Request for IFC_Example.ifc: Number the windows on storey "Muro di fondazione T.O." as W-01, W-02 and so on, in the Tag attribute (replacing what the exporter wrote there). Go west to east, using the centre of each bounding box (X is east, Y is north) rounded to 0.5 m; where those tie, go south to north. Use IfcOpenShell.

First a look at what the model holds.

```python
import ifcopenshell
import ifcopenshell.util.element
import ifcopenshell.util.placement

model = ifcopenshell.open("IFC_Example.ifc")
print(model.schema)
storey = next(s for s in model.by_type("IfcBuildingStorey") if s.Name == "Muro di fondazione T.O.")
windows = [e for e in ifcopenshell.util.element.get_decomposition(storey) if e.is_a("IfcWindow")]
for e in sorted(windows, key=lambda e: e.id()):
    origin = ifcopenshell.util.placement.get_local_placement(e.ObjectPlacement)[:3, 3]
    print(e.id(), e.Tag, e.Name, origin.round(2) + 0.0, sep=" | ")
```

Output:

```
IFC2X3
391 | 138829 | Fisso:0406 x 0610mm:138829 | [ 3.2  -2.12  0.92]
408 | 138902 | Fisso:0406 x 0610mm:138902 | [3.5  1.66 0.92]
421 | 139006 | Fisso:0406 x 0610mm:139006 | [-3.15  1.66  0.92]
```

```python
import ifcopenshell
import ifcopenshell.geom
import ifcopenshell.util.element
import ifcopenshell.util.shape

model = ifcopenshell.open("IFC_Example.ifc")
settings = ifcopenshell.geom.settings()
settings.set("use-world-coords", True)


def centre(element):
    shape = ifcopenshell.geom.create_shape(settings, element)
    return ifcopenshell.util.shape.get_bbox_centroid(shape.geometry)


storey = next(s for s in model.by_type("IfcBuildingStorey") if s.Name == "Muro di fondazione T.O.")
windows = [e for e in ifcopenshell.util.element.get_decomposition(storey) if e.is_a("IfcWindow")]

# Insertion points can sit at a corner or the storey origin, so sort by the geometry (in metres).
centres = {e: centre(e) for e in windows}
windows.sort(key=lambda e: (round(centres[e][0] / 0.5), centres[e][1]))

for i, e in enumerate(windows, start=1):
    number = f"W-{i:02d}"
    e.Tag = number
    print(e.id(), number)

model.write("IFC_Example_v2.ifc")
```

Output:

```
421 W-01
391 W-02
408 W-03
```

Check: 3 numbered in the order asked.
